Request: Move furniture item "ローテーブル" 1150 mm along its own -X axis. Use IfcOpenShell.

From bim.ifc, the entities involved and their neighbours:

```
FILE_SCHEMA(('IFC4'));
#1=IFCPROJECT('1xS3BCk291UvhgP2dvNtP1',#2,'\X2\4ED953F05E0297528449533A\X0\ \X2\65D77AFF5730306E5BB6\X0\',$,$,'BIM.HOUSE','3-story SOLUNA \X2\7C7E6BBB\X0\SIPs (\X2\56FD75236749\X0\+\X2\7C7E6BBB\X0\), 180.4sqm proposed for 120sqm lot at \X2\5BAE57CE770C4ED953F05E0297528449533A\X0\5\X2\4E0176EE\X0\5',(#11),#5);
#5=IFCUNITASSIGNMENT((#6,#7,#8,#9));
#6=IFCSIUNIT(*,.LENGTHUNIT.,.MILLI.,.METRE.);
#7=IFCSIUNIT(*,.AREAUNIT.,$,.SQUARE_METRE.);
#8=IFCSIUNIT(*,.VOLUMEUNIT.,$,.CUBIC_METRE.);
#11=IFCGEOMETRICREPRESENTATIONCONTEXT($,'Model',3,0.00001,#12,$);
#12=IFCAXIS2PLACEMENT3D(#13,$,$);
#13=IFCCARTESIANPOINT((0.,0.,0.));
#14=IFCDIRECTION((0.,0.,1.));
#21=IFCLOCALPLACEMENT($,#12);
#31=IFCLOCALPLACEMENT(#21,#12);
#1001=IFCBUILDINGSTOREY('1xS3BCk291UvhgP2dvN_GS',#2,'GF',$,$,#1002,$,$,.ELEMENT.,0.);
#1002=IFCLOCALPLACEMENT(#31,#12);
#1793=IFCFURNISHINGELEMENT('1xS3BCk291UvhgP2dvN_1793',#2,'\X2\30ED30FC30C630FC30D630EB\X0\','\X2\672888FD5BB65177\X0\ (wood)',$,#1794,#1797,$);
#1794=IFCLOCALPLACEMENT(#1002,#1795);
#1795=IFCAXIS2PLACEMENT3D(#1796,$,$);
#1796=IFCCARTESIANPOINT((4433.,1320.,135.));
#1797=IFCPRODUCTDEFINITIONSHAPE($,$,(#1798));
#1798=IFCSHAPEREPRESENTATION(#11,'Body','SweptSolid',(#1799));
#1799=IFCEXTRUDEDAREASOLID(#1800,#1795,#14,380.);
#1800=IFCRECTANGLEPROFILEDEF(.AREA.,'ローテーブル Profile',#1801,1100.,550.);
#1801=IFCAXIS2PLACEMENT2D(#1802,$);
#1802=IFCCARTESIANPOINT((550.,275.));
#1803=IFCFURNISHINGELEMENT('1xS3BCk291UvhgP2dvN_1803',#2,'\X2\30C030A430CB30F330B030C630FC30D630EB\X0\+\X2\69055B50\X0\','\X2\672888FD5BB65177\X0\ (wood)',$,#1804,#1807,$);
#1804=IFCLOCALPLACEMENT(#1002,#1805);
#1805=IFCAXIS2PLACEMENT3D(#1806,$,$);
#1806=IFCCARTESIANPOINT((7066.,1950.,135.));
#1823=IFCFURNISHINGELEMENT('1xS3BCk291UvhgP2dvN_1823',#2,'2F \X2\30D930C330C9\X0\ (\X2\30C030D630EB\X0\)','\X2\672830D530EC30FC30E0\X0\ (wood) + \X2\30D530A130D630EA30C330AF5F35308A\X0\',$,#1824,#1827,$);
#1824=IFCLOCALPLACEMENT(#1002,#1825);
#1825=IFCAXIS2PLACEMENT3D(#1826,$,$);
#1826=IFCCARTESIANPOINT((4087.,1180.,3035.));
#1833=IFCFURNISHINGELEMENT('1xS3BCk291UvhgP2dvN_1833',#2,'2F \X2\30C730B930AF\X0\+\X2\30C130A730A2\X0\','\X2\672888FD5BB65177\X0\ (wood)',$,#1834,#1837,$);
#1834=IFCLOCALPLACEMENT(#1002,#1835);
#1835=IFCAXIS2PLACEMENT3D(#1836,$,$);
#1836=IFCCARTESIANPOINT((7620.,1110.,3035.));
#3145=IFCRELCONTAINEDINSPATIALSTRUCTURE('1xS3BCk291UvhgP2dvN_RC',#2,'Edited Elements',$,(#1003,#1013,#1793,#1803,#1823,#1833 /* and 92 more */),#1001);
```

```python
import ifcopenshell
import ifcopenshell.api.geometry
import ifcopenshell.util.placement
import ifcopenshell.util.unit

model = ifcopenshell.open("bim.ifc")
unit_scale = ifcopenshell.util.unit.calculate_unit_scale(model)

item = model.by_guid("1xS3BCk291UvhgP2dvN_1793")
matrix = ifcopenshell.util.placement.get_local_placement(item.ObjectPlacement)
matrix[:3, 3] -= matrix[:3, 0] * 1.15 / unit_scale
ifcopenshell.api.geometry.edit_object_placement(model, product=item, matrix=matrix, is_si=False)

print(ifcopenshell.util.placement.get_local_placement(item.ObjectPlacement).round(3) + 0.0)

model.write("bim-out.ifc")
```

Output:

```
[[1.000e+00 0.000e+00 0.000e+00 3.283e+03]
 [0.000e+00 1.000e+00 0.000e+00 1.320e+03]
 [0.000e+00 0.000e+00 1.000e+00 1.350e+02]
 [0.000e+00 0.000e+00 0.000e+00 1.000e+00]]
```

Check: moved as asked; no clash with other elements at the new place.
